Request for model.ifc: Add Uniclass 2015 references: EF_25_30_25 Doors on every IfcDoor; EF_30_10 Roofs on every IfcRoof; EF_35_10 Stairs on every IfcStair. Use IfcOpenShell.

First a look at what the model holds.

```python
import ifcopenshell

model = ifcopenshell.open("model.ifc")
print(model.schema)
print("classifications:", [c.Name for c in model.by_type("IfcClassification")])
for ifc_class in ("IfcDoor", "IfcRoof", "IfcStair", "IfcWall", "IfcWindow"):
    print(ifc_class, len(model.by_type(ifc_class)))
```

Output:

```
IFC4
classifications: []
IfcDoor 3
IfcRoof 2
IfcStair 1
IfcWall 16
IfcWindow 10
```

```python
import ifcopenshell
import ifcopenshell.api.classification

model = ifcopenshell.open("model.ifc")

system = ifcopenshell.api.classification.add_classification(model, classification="Uniclass 2015")

codes = {
    "IfcDoor": ("EF_25_30_25", "Doors"),
    "IfcRoof": ("EF_30_10", "Roofs"),
    "IfcStair": ("EF_35_10", "Stairs"),
}
for ifc_class, (code, name) in codes.items():
    products = model.by_type(ifc_class)
    ifcopenshell.api.classification.add_reference(
        model, products=products, classification=system, identification=code, name=name
    )
    print(code, len(products))

model.write("model_edited.ifc")
```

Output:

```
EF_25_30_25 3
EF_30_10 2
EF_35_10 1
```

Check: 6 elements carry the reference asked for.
